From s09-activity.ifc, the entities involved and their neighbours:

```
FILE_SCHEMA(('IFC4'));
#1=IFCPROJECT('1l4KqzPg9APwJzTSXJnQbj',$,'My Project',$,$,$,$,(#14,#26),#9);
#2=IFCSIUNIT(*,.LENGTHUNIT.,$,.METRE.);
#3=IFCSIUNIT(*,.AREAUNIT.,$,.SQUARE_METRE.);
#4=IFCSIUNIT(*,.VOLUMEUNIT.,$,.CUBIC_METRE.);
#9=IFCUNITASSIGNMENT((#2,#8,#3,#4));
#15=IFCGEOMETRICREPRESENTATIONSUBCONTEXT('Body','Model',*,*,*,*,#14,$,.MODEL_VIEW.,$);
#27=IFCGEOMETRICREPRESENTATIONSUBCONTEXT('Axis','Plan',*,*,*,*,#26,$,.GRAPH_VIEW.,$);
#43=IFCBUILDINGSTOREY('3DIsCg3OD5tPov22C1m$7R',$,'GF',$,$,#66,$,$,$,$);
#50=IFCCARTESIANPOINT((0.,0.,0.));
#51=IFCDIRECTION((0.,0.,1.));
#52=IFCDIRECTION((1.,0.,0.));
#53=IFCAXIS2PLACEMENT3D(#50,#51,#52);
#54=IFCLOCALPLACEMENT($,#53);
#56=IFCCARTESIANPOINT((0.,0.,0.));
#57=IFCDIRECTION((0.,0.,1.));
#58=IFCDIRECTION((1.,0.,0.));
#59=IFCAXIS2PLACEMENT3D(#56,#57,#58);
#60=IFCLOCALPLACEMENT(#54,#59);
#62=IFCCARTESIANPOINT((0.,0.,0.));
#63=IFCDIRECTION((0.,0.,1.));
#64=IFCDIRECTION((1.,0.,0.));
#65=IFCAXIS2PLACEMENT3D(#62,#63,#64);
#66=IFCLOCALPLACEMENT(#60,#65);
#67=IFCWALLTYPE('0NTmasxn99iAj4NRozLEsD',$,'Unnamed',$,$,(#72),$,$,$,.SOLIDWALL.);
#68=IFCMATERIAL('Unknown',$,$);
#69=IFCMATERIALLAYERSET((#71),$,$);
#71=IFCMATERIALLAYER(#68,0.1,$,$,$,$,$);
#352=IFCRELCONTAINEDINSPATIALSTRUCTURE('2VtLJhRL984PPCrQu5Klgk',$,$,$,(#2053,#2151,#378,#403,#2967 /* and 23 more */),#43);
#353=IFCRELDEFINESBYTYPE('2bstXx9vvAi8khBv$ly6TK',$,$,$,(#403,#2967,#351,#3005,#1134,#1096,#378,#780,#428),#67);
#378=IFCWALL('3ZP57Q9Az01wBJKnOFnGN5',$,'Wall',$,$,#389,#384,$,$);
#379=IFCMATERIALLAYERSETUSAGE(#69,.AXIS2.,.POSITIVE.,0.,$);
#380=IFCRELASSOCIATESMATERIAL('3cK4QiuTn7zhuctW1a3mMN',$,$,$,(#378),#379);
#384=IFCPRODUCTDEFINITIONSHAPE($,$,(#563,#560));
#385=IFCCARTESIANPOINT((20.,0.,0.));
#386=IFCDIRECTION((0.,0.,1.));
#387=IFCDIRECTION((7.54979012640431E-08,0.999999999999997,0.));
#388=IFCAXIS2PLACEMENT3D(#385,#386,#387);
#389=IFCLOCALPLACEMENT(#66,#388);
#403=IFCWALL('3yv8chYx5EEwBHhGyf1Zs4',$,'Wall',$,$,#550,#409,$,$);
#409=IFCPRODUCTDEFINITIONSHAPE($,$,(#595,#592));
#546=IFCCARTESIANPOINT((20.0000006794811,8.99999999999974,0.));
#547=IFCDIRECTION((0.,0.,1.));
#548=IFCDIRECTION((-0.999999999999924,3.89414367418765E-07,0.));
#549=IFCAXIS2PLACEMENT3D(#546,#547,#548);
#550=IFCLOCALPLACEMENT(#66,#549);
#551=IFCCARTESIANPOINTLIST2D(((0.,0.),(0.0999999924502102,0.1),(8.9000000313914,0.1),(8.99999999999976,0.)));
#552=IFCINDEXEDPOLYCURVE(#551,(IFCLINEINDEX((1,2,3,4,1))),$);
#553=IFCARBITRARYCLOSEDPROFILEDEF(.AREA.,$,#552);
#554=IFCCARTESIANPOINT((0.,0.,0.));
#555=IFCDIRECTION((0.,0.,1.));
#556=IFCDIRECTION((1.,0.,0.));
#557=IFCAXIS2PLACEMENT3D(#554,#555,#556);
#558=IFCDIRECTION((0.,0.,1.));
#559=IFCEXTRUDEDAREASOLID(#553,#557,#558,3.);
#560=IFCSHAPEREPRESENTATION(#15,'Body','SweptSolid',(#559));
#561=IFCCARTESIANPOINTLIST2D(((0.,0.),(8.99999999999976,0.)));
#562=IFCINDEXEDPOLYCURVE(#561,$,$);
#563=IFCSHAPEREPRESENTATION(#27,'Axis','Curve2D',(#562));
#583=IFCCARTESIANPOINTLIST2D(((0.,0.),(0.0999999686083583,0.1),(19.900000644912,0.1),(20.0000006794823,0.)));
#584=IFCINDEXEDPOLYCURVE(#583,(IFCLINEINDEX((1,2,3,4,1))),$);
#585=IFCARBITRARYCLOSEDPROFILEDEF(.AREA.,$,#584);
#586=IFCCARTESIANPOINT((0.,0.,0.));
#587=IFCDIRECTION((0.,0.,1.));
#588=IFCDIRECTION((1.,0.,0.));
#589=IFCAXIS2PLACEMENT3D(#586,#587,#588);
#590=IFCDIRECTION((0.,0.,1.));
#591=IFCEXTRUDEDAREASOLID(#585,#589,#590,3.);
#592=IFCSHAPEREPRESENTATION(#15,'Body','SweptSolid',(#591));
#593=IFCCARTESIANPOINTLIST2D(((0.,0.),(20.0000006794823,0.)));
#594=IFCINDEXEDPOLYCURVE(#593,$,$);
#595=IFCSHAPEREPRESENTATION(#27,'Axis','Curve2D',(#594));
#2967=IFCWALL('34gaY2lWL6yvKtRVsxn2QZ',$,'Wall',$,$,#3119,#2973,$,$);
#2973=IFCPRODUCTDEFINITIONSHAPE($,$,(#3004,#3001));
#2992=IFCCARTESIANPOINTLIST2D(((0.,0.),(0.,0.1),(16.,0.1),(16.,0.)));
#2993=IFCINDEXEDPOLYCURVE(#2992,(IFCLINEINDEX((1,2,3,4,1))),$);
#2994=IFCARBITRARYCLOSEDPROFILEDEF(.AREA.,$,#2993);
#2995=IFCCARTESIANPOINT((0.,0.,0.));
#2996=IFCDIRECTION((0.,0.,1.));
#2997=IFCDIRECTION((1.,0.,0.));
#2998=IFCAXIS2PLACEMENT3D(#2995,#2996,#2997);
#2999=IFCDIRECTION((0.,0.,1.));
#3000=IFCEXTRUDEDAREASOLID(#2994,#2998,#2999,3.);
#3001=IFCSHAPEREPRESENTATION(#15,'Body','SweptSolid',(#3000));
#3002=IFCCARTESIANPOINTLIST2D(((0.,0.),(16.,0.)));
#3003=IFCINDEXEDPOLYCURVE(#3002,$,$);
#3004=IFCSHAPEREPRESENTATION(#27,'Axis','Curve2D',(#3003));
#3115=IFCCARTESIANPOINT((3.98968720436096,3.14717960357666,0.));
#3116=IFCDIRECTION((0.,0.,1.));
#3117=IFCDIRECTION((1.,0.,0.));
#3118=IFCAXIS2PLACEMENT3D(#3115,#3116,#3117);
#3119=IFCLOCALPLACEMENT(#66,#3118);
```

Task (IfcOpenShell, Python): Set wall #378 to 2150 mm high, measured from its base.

```python
import ifcopenshell
import ifcopenshell.geom
import ifcopenshell.util.representation
import ifcopenshell.util.shape

model = ifcopenshell.open("s09-activity.ifc")
settings = ifcopenshell.geom.settings()


def volume(element):
    """Net volume in cubic metres, openings subtracted."""
    shape = ifcopenshell.geom.create_shape(settings, element)
    return ifcopenshell.util.shape.get_volume(shape.geometry)


wall = model.by_guid("3ZP57Q9Az01wBJKnOFnGN5")
before = volume(wall)

body = ifcopenshell.util.representation.get_representation(wall, "Model", "Body")
solid = body.Items[0]
old_height = solid.Depth
solid.Depth = 2.15
after = volume(wall)

print(f"height {old_height:g} -> {solid.Depth:g}, volume {before:.3f} -> {after:.3f} m3")

model.write("s09-activity_updated.ifc")
```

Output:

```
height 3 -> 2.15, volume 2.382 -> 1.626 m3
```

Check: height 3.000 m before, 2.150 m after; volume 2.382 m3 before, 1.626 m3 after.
